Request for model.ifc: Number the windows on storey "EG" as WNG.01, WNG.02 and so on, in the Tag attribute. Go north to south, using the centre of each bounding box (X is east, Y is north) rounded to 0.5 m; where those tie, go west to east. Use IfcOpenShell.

First a look at what the model holds.

```python
import ifcopenshell
import ifcopenshell.util.element
import ifcopenshell.util.placement

model = ifcopenshell.open("model.ifc")
print(model.schema)
storey = next(s for s in model.by_type("IfcBuildingStorey") if s.Name == "EG")
windows = [e for e in ifcopenshell.util.element.get_decomposition(storey) if e.is_a("IfcWindow")]
for e in sorted(windows, key=lambda e: e.id()):
    origin = ifcopenshell.util.placement.get_local_placement(e.ObjectPlacement)[:3, 3]
    print(e.id(), e.Tag, e.Name, origin.round(2) + 0.0, sep=" | ")
```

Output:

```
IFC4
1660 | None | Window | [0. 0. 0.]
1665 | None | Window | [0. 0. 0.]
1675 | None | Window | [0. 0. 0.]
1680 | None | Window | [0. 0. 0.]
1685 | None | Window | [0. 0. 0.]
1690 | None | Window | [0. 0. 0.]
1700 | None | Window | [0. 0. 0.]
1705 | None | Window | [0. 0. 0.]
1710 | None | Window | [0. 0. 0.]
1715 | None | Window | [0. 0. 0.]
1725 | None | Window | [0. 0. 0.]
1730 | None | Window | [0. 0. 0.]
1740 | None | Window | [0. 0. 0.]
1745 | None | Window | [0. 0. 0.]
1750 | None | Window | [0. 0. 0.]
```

```python
import ifcopenshell
import ifcopenshell.geom
import ifcopenshell.util.element
import ifcopenshell.util.shape

model = ifcopenshell.open("model.ifc")
settings = ifcopenshell.geom.settings()
settings.set("use-world-coords", True)


def centre(element):
    shape = ifcopenshell.geom.create_shape(settings, element)
    return ifcopenshell.util.shape.get_bbox_centroid(shape.geometry)


storey = next(s for s in model.by_type("IfcBuildingStorey") if s.Name == "EG")
windows = [e for e in ifcopenshell.util.element.get_decomposition(storey) if e.is_a("IfcWindow")]

# Insertion points can sit at a corner or the storey origin, so sort by the geometry (in metres).
centres = {e: centre(e) for e in windows}
windows.sort(key=lambda e: (-round(centres[e][1] / 0.5), centres[e][0]))

for i, e in enumerate(windows, start=1):
    number = f"WNG.{i:02d}"
    e.Tag = number
    print(e.id(), number)

model.write("model_edited.ifc")
```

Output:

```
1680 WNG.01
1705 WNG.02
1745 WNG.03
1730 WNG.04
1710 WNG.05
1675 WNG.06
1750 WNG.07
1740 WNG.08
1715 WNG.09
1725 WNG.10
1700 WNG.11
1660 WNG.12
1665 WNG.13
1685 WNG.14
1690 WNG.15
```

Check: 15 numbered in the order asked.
